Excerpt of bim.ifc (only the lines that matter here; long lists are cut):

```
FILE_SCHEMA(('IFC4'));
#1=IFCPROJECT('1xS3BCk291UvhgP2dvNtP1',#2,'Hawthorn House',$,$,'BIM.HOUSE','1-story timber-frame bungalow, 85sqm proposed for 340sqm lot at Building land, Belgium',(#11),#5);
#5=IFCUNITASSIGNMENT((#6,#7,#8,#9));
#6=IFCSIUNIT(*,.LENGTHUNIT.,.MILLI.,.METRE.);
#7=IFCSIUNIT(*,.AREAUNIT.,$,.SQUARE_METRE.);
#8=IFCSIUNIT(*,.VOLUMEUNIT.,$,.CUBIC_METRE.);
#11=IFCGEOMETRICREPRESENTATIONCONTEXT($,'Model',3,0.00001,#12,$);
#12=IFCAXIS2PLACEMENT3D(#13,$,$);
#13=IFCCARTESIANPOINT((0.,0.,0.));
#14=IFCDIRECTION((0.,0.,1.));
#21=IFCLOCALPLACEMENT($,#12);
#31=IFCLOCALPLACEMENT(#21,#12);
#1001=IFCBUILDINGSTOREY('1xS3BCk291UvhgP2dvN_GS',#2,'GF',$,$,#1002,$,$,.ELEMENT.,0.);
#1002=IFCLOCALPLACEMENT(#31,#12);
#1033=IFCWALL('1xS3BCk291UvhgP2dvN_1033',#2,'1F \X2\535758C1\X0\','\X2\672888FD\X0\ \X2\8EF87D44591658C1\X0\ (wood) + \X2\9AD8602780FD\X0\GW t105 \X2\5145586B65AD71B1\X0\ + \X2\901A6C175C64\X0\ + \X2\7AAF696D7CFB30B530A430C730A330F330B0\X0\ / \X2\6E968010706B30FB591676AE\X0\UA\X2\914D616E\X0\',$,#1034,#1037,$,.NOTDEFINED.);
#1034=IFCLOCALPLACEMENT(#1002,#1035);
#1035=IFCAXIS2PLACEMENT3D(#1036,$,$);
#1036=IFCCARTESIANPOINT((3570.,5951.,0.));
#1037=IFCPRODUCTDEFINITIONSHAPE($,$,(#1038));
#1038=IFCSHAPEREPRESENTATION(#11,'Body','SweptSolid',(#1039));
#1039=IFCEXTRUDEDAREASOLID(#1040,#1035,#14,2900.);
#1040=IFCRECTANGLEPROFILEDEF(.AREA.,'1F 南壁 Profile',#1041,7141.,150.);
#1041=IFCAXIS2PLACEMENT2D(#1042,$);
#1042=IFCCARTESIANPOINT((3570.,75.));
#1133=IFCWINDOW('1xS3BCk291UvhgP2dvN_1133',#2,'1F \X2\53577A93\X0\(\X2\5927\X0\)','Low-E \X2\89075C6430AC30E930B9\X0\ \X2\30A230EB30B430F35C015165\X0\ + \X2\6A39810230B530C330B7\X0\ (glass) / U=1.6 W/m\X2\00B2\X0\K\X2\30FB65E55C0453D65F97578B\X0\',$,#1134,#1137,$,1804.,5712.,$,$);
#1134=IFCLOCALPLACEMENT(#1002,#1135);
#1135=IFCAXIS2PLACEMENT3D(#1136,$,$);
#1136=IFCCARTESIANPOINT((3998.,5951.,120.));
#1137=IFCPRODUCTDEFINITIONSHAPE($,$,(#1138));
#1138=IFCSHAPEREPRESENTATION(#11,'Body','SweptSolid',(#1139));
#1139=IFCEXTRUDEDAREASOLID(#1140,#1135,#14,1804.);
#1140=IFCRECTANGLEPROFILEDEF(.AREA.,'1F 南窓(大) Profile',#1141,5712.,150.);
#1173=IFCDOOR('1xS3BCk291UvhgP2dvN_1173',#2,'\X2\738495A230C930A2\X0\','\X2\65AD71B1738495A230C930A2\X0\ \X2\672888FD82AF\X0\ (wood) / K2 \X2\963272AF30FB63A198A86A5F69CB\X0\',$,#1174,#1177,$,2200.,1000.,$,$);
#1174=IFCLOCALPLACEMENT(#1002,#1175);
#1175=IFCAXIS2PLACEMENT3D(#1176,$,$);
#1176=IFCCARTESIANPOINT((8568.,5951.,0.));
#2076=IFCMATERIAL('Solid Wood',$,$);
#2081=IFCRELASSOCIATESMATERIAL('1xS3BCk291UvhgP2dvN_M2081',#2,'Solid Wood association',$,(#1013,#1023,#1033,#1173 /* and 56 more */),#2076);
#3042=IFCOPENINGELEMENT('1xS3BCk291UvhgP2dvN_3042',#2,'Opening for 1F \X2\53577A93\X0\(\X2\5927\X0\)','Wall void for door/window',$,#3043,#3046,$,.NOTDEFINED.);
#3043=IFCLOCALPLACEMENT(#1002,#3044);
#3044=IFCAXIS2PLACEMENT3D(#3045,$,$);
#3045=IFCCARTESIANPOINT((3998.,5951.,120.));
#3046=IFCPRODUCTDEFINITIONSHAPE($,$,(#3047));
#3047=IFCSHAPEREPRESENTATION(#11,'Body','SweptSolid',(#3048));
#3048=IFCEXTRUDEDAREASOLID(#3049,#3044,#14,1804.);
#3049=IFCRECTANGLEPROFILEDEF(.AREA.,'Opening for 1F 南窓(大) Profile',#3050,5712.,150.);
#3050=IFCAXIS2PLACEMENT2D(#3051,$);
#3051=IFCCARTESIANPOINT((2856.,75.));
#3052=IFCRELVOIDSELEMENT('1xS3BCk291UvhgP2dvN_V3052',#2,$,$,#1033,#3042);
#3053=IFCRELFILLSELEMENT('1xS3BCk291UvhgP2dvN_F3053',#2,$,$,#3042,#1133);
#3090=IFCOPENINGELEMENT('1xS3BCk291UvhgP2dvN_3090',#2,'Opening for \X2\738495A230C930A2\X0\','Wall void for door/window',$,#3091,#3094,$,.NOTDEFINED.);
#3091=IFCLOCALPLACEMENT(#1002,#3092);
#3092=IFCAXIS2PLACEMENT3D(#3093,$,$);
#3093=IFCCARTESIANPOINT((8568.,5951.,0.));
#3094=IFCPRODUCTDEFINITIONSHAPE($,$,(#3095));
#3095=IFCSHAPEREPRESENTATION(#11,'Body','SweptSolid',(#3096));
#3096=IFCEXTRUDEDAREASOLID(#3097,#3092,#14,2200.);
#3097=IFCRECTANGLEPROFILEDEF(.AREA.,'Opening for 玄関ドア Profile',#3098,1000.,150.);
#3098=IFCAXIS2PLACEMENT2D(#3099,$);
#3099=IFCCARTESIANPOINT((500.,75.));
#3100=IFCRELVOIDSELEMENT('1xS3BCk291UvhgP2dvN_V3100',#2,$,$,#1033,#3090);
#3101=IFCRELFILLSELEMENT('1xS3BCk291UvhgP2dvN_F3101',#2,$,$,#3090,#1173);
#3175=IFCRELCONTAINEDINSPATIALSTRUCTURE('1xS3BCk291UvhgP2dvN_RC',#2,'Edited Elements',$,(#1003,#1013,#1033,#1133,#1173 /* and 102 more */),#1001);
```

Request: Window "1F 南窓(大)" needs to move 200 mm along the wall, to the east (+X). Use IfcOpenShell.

```python
import ifcopenshell
import ifcopenshell.api.geometry
import ifcopenshell.util.placement
import ifcopenshell.util.unit

model = ifcopenshell.open("bim.ifc")
unit_scale = ifcopenshell.util.unit.calculate_unit_scale(model)

window = model.by_guid("1xS3BCk291UvhgP2dvN_1133")
opening = window.FillsVoids[0].RelatingOpeningElement
wall = opening.VoidsElements[0].RelatingBuildingElement

wall_matrix = ifcopenshell.util.placement.get_local_placement(wall.ObjectPlacement)
shift = wall_matrix[:3, 0] * 0.2 / unit_scale
before = ifcopenshell.util.placement.get_local_placement(window.ObjectPlacement)[:3, 3].copy()

# The window is not placed relative to its opening, so move both.
for product in (opening, window):
    matrix = ifcopenshell.util.placement.get_local_placement(product.ObjectPlacement)
    matrix[:3, 3] += shift
    ifcopenshell.api.geometry.edit_object_placement(model, product=product, matrix=matrix, is_si=False)

after = ifcopenshell.util.placement.get_local_placement(window.ObjectPlacement)[:3, 3]
print("window moved by", (after - before).round(3) + 0.0)

model.write("bim_rev.ifc")
```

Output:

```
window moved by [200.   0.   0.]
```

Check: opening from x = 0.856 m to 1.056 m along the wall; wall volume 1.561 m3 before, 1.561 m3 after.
